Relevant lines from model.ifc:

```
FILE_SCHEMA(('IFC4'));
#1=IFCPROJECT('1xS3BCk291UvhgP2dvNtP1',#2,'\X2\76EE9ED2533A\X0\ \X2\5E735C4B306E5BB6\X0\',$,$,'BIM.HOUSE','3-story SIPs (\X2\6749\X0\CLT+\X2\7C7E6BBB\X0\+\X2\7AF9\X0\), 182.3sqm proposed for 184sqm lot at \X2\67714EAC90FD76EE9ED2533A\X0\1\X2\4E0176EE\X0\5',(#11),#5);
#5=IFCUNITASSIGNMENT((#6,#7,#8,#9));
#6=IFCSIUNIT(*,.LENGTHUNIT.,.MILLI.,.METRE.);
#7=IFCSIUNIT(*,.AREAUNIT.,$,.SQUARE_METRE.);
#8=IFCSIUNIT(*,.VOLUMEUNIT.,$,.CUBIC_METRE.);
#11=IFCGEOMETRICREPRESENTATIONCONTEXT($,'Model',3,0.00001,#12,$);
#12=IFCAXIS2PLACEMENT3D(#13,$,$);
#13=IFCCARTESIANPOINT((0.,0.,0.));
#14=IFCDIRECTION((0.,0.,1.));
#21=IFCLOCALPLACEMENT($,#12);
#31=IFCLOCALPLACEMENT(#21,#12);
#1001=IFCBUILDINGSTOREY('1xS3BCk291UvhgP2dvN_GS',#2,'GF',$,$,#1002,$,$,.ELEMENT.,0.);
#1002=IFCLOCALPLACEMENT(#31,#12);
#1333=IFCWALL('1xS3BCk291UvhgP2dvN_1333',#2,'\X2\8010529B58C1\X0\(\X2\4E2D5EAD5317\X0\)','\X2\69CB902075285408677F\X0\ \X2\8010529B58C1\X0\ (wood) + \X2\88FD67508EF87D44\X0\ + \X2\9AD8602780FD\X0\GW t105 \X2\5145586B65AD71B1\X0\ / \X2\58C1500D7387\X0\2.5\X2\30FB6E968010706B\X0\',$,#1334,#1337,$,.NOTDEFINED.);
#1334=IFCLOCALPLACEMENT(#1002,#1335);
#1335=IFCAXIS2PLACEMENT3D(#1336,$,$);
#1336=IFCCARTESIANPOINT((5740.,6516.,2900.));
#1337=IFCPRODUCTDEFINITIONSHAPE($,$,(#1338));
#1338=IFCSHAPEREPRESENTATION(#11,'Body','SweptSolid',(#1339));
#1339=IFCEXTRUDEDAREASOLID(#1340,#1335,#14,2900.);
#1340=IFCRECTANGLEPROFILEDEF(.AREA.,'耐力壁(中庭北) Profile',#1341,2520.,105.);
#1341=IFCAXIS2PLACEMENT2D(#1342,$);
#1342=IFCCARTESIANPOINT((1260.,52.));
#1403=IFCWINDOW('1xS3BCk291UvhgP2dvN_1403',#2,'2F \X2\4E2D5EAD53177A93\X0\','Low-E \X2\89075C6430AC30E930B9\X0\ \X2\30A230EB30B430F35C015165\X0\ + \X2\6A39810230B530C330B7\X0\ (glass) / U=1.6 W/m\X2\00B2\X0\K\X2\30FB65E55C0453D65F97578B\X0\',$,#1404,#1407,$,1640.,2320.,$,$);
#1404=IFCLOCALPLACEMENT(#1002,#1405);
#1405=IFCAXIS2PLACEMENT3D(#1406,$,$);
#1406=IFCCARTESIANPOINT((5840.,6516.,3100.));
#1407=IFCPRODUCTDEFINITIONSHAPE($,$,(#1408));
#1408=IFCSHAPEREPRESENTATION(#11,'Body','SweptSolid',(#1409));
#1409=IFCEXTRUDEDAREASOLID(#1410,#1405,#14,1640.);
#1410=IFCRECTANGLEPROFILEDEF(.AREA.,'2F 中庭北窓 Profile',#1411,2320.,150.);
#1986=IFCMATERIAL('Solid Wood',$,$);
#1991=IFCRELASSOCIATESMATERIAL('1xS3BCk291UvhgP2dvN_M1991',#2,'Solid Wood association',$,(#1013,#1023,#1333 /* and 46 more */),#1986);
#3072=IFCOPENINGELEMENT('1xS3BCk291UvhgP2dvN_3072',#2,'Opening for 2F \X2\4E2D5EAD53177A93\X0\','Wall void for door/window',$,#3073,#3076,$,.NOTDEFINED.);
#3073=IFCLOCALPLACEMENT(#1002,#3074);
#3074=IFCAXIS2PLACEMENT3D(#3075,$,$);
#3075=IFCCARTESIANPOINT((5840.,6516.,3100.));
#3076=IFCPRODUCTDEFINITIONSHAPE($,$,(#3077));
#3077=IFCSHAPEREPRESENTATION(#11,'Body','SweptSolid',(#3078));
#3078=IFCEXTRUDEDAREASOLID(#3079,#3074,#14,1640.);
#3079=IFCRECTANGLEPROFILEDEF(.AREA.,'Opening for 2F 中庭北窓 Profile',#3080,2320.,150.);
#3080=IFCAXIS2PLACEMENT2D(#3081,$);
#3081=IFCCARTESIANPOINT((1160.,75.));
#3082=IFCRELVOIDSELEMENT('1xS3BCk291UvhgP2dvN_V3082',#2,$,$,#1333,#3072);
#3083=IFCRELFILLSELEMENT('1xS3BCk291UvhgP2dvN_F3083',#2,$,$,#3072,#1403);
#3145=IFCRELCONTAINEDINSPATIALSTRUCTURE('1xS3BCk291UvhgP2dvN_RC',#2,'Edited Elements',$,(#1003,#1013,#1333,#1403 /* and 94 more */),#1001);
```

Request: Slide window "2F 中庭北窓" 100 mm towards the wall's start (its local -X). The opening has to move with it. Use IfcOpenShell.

```python
import ifcopenshell
import ifcopenshell.api.geometry
import ifcopenshell.util.placement

model = ifcopenshell.open("model.ifc")

window = model.by_guid("1xS3BCk291UvhgP2dvN_1403")
opening = window.FillsVoids[0].RelatingOpeningElement
wall = opening.VoidsElements[0].RelatingBuildingElement

wall_matrix = ifcopenshell.util.placement.get_local_placement(wall.ObjectPlacement)
shift = wall_matrix[:3, 0] * -100.0
before = ifcopenshell.util.placement.get_local_placement(window.ObjectPlacement)[:3, 3].copy()

# The window is not placed relative to its opening, so move both.
for product in (opening, window):
    matrix = ifcopenshell.util.placement.get_local_placement(product.ObjectPlacement)
    matrix[:3, 3] += shift
    ifcopenshell.api.geometry.edit_object_placement(model, product=product, matrix=matrix, is_si=False)

after = ifcopenshell.util.placement.get_local_placement(window.ObjectPlacement)[:3, 3]
print("window moved by", (after - before).round(3) + 0.0)

model.write("model_updated.ifc")
```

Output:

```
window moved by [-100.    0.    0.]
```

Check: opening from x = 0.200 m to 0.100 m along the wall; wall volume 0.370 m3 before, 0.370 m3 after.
